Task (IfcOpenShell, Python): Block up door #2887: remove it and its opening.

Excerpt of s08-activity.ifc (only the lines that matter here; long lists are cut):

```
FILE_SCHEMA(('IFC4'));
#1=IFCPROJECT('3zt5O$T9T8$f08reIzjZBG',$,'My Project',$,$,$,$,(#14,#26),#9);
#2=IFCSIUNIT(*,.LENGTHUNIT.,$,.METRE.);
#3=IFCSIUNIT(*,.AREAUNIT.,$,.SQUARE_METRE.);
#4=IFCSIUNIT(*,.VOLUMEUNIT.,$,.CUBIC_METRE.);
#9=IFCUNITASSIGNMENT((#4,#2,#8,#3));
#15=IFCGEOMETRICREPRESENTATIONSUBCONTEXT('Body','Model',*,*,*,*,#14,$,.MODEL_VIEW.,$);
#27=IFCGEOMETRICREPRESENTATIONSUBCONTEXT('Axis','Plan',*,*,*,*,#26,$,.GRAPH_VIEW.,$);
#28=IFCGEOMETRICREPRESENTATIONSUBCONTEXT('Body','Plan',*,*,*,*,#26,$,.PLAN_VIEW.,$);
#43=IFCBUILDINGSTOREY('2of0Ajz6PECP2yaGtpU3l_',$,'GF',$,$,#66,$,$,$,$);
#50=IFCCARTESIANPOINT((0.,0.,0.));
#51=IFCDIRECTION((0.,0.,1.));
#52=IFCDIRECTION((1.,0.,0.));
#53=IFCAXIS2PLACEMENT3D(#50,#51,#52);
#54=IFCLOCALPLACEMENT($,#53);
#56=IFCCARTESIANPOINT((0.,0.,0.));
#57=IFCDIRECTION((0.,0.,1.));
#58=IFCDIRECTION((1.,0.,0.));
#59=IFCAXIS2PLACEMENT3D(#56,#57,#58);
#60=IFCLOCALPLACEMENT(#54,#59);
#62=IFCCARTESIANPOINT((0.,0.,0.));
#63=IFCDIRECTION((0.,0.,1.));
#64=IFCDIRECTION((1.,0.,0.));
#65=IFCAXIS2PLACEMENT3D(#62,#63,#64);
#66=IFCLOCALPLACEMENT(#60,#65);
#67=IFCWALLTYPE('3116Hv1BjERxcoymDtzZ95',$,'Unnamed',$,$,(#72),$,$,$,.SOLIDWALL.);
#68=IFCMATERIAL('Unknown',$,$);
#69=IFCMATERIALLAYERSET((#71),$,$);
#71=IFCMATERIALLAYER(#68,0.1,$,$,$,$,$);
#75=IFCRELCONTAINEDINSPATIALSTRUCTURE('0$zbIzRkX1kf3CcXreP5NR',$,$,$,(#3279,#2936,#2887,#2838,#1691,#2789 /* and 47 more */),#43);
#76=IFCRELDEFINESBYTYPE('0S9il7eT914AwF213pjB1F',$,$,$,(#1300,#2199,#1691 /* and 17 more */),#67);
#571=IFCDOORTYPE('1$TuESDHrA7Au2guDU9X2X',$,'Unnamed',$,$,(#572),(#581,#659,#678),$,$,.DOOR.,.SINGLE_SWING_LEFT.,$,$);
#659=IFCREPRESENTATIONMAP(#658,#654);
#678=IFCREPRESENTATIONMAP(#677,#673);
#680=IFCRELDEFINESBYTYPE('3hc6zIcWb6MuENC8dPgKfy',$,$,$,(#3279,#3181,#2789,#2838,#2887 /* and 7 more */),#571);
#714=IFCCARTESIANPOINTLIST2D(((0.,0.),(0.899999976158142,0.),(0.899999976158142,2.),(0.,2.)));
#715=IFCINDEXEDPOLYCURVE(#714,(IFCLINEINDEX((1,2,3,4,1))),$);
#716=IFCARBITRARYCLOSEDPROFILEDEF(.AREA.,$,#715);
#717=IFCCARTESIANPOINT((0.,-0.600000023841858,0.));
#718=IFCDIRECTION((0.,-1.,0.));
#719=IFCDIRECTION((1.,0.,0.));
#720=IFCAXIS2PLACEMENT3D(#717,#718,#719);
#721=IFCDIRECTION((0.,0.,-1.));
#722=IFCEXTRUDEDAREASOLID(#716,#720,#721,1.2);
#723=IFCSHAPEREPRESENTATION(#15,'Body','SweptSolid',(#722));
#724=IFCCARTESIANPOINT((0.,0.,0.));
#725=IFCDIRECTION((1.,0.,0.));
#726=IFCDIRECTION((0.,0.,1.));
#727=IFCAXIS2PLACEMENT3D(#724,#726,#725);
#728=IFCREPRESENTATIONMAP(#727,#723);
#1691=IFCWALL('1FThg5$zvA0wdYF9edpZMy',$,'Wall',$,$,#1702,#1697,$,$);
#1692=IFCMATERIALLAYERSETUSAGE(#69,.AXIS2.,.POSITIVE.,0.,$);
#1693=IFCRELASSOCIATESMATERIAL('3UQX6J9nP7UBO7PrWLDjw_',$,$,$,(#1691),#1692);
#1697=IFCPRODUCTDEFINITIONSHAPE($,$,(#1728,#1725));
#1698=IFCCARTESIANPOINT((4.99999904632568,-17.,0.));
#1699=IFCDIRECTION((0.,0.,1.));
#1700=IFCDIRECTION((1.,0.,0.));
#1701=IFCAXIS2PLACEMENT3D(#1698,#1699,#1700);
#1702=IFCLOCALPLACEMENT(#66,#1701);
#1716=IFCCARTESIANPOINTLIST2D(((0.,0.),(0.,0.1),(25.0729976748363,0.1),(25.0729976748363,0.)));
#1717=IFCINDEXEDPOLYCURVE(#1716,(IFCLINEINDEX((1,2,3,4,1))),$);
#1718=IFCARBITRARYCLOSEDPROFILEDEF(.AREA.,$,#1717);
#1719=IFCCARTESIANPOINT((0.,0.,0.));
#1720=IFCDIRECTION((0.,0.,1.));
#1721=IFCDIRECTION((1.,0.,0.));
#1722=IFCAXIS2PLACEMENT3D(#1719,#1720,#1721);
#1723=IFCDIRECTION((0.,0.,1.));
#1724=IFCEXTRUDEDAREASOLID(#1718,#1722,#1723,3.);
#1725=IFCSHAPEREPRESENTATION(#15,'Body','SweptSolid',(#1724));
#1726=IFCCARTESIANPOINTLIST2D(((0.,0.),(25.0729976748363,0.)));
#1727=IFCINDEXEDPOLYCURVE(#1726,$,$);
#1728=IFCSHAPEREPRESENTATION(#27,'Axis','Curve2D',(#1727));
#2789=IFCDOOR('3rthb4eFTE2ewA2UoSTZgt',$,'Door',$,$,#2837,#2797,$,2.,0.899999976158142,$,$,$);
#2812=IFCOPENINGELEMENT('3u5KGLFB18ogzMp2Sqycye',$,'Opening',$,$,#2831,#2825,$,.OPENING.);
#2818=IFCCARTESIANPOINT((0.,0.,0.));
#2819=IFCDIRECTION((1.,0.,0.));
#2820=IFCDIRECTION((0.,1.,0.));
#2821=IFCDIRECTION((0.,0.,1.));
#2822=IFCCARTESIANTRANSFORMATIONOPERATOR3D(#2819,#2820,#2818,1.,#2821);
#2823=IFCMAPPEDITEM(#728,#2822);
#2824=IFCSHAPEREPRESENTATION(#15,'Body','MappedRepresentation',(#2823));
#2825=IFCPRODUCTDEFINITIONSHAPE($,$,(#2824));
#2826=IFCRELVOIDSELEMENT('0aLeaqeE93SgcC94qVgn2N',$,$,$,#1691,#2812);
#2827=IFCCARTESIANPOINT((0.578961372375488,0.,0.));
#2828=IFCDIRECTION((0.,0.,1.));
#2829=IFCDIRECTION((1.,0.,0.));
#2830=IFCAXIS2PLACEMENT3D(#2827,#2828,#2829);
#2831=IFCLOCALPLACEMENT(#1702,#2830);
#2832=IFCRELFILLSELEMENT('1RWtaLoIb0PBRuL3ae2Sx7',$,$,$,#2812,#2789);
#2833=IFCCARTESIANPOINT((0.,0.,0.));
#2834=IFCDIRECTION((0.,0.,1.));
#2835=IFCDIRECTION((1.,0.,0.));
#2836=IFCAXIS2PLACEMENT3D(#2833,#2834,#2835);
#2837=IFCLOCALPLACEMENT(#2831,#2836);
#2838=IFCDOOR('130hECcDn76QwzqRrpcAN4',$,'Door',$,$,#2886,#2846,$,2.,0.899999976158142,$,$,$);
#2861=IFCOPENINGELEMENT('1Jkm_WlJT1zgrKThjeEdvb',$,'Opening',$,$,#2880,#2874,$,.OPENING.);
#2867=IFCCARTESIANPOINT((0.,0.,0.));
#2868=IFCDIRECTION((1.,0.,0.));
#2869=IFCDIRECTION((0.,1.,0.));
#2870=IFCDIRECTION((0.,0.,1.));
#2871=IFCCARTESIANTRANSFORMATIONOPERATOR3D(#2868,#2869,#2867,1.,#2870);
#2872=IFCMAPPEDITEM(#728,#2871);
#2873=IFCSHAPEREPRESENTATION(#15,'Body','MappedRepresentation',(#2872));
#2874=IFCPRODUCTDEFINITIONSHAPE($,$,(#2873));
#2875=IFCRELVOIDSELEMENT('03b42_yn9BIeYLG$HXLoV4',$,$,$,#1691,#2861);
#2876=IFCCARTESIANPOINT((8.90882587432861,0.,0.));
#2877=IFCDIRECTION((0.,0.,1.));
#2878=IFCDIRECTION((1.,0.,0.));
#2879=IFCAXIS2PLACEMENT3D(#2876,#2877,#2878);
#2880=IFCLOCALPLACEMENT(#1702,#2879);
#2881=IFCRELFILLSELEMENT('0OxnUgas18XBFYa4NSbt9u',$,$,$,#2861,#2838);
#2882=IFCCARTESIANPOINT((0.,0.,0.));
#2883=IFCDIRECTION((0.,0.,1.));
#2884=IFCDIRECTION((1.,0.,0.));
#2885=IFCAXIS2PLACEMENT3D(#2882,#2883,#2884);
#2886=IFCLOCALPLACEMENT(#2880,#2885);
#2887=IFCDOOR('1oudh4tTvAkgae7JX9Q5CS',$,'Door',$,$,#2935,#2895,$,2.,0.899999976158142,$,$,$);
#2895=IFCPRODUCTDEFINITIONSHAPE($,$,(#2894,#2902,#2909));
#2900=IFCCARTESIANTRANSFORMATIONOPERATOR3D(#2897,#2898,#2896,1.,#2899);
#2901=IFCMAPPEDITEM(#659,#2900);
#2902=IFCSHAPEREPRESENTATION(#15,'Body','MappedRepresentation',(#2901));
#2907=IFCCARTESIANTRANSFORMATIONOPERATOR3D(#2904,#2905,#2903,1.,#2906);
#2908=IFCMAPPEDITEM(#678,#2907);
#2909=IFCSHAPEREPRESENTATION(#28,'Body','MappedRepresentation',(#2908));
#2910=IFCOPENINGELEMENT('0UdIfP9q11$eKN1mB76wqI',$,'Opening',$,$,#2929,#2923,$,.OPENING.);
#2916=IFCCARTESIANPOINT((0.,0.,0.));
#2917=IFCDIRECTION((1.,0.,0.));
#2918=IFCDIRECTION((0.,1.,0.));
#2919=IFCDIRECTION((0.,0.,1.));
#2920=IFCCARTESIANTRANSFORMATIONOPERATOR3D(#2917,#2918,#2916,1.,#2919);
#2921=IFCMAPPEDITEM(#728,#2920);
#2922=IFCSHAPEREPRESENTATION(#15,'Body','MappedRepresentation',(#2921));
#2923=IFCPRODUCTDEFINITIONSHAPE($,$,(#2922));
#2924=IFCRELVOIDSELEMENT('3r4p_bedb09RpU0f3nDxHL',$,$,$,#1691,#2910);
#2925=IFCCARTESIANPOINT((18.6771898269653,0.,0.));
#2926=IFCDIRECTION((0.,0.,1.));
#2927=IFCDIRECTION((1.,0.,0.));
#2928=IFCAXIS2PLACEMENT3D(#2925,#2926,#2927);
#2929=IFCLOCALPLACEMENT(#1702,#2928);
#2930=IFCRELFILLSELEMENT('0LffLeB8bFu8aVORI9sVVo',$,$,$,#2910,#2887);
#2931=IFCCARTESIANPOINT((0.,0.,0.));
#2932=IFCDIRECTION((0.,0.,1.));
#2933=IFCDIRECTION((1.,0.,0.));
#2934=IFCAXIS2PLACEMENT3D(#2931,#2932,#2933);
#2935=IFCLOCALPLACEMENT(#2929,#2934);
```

```python
import ifcopenshell
import ifcopenshell.api.feature
import ifcopenshell.api.root
import ifcopenshell.geom
import ifcopenshell.util.shape

model = ifcopenshell.open("s08-activity.ifc")
settings = ifcopenshell.geom.settings()


def volume(element):
    """Net volume in cubic metres, openings subtracted."""
    shape = ifcopenshell.geom.create_shape(settings, element)
    return ifcopenshell.util.shape.get_volume(shape.geometry)


door = model.by_guid("1oudh4tTvAkgae7JX9Q5CS")
opening = door.FillsVoids[0].RelatingOpeningElement
wall = opening.VoidsElements[0].RelatingBuildingElement
before = volume(wall)

ifcopenshell.api.root.remove_product(model, product=door)
ifcopenshell.api.feature.remove_feature(model, feature=opening)

after = volume(wall)

print(f"wall volume {before:.3f} -> {after:.3f} m3")

model.write("s08-activity_updated.ifc")
```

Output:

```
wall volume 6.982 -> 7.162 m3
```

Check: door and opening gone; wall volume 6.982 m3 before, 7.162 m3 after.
